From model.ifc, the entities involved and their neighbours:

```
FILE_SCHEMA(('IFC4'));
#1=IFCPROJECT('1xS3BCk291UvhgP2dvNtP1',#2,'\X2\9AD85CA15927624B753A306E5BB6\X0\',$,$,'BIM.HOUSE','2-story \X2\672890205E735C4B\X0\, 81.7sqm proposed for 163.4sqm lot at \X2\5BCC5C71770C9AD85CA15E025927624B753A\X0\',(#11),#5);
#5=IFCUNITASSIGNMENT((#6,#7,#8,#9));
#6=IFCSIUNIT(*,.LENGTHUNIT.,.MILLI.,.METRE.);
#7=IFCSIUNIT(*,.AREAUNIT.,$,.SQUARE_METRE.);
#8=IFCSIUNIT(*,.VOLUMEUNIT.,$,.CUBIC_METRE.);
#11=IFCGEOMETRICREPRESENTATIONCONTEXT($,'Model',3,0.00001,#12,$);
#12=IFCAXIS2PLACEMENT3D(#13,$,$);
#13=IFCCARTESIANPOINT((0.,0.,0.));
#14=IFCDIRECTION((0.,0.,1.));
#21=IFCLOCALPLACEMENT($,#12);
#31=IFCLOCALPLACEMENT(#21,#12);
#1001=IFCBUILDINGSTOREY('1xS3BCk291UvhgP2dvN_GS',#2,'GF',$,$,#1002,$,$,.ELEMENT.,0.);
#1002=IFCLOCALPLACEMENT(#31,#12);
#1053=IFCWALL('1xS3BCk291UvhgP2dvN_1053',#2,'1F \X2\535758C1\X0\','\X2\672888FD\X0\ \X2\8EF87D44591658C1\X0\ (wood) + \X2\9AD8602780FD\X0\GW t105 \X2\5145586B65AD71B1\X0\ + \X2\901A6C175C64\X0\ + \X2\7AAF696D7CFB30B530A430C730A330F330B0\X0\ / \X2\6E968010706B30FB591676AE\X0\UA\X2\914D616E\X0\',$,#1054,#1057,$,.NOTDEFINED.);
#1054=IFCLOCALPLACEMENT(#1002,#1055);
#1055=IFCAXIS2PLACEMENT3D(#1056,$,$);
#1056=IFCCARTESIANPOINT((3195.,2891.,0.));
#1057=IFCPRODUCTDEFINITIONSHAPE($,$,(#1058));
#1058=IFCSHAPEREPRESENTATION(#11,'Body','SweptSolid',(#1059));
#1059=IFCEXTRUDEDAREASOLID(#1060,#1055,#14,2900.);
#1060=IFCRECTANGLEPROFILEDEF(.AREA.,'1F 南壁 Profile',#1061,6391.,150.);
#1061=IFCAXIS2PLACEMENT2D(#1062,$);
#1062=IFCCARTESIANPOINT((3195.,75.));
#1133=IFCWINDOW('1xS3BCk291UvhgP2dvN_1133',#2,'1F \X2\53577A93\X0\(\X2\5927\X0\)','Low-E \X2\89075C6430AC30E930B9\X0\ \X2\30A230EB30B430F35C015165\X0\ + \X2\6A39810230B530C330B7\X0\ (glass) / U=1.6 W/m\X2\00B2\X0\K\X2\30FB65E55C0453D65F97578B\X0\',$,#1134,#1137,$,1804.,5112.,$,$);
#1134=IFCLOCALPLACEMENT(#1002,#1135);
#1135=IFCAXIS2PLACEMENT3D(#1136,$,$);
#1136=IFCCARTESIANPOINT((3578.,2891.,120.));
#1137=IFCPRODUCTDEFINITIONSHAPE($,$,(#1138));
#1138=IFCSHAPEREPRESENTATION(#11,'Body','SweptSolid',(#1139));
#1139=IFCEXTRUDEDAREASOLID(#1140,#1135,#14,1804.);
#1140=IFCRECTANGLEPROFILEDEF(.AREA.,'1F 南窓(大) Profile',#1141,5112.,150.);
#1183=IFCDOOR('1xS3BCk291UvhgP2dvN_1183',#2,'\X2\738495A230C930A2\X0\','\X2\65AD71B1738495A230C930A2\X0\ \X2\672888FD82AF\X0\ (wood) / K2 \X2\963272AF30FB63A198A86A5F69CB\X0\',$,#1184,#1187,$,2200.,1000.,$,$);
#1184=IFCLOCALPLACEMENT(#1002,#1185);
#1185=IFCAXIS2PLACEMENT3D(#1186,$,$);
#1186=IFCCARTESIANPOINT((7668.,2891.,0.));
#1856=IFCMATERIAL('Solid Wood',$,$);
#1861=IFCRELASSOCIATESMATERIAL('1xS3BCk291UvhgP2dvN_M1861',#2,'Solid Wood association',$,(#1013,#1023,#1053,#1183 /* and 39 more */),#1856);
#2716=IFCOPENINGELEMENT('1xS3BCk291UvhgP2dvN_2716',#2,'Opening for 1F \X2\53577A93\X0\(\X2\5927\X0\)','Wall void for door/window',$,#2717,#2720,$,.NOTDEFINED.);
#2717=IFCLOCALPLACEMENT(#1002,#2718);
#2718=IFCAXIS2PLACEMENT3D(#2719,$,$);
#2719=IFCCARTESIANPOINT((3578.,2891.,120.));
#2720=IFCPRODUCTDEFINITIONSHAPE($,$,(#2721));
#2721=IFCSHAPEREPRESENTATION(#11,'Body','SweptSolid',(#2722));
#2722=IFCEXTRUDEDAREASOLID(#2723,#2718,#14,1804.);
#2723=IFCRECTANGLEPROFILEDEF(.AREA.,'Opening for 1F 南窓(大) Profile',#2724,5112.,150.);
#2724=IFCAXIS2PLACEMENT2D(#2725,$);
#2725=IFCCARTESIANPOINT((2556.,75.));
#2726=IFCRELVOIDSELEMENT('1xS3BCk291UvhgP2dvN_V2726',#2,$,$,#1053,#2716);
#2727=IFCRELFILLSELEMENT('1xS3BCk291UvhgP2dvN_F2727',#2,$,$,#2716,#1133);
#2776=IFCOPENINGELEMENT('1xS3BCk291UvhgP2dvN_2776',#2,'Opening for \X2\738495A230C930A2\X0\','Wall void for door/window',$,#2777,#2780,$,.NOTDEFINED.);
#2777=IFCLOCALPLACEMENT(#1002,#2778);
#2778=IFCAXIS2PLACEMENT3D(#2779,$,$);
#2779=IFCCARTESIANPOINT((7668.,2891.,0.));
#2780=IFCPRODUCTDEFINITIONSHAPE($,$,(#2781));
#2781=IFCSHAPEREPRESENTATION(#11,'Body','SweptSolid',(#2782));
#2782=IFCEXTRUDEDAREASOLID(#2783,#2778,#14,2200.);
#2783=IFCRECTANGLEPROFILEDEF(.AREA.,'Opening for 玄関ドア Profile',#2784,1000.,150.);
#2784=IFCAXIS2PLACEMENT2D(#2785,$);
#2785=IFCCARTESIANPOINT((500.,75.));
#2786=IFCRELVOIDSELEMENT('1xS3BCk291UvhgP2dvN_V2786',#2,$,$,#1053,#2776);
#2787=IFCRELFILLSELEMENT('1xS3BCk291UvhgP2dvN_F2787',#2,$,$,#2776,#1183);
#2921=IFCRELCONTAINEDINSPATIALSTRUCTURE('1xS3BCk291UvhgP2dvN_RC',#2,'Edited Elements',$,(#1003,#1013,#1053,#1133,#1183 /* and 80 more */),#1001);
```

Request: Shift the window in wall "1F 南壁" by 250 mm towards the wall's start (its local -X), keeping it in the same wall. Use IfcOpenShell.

```python
import ifcopenshell
import ifcopenshell.api.geometry
import ifcopenshell.util.placement
import ifcopenshell.util.unit

model = ifcopenshell.open("model.ifc")
unit_scale = ifcopenshell.util.unit.calculate_unit_scale(model)

window = model.by_guid("1xS3BCk291UvhgP2dvN_1133")
opening = window.FillsVoids[0].RelatingOpeningElement
wall = opening.VoidsElements[0].RelatingBuildingElement

wall_matrix = ifcopenshell.util.placement.get_local_placement(wall.ObjectPlacement)
shift = wall_matrix[:3, 0] * -0.25 / unit_scale
before = ifcopenshell.util.placement.get_local_placement(window.ObjectPlacement)[:3, 3].copy()

# The window is not placed relative to its opening, so move both.
for product in (opening, window):
    matrix = ifcopenshell.util.placement.get_local_placement(product.ObjectPlacement)
    matrix[:3, 3] += shift
    ifcopenshell.api.geometry.edit_object_placement(model, product=product, matrix=matrix, is_si=False)

after = ifcopenshell.util.placement.get_local_placement(window.ObjectPlacement)[:3, 3]
print("window moved by", (after - before).round(3) + 0.0)

model.write("model_rev.ifc")
```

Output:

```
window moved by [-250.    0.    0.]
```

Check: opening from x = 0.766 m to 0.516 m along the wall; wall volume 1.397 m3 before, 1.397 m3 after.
